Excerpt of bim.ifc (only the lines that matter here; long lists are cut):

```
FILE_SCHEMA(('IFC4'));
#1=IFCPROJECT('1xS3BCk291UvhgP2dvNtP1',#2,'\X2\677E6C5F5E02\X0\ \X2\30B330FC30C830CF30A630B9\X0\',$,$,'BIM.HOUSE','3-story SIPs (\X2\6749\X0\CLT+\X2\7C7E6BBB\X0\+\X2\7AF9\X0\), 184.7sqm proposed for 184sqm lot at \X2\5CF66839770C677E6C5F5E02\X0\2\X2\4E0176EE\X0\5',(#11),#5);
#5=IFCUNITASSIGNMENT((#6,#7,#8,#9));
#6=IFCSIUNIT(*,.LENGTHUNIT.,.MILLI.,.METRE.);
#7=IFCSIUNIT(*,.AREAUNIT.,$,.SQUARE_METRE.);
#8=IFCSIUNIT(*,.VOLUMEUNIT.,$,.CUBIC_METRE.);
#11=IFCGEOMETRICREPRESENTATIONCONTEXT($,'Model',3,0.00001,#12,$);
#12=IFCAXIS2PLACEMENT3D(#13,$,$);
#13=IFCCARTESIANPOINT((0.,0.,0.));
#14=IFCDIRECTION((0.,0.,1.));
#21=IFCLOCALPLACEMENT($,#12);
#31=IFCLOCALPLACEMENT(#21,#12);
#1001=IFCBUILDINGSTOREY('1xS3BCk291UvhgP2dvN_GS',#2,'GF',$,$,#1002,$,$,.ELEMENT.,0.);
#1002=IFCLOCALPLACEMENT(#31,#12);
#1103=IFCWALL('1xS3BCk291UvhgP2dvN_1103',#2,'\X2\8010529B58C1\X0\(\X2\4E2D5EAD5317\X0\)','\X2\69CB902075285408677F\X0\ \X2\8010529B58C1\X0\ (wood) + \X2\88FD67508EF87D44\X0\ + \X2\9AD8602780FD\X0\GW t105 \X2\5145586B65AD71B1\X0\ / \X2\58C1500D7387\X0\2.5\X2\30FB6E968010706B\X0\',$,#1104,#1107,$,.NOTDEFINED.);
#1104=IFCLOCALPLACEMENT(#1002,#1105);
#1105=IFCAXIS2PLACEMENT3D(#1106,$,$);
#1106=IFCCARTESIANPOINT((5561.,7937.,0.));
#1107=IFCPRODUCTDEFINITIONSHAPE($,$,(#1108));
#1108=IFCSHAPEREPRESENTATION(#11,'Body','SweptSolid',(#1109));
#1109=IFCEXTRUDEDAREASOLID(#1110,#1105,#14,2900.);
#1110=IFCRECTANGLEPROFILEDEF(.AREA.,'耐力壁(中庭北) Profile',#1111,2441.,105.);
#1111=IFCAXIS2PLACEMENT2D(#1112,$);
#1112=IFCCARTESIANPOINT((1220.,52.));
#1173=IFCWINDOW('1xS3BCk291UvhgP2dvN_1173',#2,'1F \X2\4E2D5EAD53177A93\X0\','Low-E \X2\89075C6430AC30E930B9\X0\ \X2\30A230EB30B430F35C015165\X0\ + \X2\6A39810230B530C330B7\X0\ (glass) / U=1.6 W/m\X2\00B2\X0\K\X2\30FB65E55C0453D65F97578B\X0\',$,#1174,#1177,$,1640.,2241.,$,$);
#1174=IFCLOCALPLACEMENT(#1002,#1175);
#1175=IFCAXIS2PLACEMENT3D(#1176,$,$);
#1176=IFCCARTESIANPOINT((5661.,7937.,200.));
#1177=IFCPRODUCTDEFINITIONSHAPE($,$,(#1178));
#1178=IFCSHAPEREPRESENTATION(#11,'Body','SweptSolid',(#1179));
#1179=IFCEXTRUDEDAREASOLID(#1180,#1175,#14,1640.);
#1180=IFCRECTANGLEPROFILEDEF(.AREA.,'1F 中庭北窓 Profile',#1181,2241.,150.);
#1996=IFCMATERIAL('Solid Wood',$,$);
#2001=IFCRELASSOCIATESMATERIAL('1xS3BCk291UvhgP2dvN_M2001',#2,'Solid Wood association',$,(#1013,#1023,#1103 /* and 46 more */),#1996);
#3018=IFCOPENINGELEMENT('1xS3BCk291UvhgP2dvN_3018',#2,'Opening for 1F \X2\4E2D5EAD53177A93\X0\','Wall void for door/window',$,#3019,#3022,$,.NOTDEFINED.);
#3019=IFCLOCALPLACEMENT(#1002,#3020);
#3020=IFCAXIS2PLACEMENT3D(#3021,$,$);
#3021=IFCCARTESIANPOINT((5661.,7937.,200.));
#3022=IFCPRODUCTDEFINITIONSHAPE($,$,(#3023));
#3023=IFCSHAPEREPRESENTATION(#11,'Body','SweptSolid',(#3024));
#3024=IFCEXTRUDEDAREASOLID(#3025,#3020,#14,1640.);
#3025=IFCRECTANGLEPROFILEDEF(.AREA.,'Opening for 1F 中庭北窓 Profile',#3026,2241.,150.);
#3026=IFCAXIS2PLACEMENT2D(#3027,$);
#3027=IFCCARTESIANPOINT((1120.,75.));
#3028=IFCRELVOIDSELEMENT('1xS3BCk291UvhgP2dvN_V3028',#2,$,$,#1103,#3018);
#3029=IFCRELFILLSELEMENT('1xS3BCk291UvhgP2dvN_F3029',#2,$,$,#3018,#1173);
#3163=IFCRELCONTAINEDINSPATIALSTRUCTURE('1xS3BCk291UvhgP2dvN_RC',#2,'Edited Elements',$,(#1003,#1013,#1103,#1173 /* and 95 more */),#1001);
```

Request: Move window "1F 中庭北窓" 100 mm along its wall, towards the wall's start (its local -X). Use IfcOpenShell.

```python
import ifcopenshell
import ifcopenshell.api.geometry
import ifcopenshell.util.placement
import ifcopenshell.util.unit

model = ifcopenshell.open("bim.ifc")
unit_scale = ifcopenshell.util.unit.calculate_unit_scale(model)

window = model.by_guid("1xS3BCk291UvhgP2dvN_1173")
opening = window.FillsVoids[0].RelatingOpeningElement
wall = opening.VoidsElements[0].RelatingBuildingElement

wall_matrix = ifcopenshell.util.placement.get_local_placement(wall.ObjectPlacement)
shift = wall_matrix[:3, 0] * -0.1 / unit_scale
before = ifcopenshell.util.placement.get_local_placement(window.ObjectPlacement)[:3, 3].copy()

# The window is not placed relative to its opening, so move both.
for product in (opening, window):
    matrix = ifcopenshell.util.placement.get_local_placement(product.ObjectPlacement)
    matrix[:3, 3] += shift
    ifcopenshell.api.geometry.edit_object_placement(model, product=product, matrix=matrix, is_si=False)

after = ifcopenshell.util.placement.get_local_placement(window.ObjectPlacement)[:3, 3]
print("window moved by", (after - before).round(3) + 0.0)

model.write("bim-out.ifc")
```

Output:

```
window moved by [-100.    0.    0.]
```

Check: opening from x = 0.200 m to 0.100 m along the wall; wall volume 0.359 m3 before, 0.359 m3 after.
